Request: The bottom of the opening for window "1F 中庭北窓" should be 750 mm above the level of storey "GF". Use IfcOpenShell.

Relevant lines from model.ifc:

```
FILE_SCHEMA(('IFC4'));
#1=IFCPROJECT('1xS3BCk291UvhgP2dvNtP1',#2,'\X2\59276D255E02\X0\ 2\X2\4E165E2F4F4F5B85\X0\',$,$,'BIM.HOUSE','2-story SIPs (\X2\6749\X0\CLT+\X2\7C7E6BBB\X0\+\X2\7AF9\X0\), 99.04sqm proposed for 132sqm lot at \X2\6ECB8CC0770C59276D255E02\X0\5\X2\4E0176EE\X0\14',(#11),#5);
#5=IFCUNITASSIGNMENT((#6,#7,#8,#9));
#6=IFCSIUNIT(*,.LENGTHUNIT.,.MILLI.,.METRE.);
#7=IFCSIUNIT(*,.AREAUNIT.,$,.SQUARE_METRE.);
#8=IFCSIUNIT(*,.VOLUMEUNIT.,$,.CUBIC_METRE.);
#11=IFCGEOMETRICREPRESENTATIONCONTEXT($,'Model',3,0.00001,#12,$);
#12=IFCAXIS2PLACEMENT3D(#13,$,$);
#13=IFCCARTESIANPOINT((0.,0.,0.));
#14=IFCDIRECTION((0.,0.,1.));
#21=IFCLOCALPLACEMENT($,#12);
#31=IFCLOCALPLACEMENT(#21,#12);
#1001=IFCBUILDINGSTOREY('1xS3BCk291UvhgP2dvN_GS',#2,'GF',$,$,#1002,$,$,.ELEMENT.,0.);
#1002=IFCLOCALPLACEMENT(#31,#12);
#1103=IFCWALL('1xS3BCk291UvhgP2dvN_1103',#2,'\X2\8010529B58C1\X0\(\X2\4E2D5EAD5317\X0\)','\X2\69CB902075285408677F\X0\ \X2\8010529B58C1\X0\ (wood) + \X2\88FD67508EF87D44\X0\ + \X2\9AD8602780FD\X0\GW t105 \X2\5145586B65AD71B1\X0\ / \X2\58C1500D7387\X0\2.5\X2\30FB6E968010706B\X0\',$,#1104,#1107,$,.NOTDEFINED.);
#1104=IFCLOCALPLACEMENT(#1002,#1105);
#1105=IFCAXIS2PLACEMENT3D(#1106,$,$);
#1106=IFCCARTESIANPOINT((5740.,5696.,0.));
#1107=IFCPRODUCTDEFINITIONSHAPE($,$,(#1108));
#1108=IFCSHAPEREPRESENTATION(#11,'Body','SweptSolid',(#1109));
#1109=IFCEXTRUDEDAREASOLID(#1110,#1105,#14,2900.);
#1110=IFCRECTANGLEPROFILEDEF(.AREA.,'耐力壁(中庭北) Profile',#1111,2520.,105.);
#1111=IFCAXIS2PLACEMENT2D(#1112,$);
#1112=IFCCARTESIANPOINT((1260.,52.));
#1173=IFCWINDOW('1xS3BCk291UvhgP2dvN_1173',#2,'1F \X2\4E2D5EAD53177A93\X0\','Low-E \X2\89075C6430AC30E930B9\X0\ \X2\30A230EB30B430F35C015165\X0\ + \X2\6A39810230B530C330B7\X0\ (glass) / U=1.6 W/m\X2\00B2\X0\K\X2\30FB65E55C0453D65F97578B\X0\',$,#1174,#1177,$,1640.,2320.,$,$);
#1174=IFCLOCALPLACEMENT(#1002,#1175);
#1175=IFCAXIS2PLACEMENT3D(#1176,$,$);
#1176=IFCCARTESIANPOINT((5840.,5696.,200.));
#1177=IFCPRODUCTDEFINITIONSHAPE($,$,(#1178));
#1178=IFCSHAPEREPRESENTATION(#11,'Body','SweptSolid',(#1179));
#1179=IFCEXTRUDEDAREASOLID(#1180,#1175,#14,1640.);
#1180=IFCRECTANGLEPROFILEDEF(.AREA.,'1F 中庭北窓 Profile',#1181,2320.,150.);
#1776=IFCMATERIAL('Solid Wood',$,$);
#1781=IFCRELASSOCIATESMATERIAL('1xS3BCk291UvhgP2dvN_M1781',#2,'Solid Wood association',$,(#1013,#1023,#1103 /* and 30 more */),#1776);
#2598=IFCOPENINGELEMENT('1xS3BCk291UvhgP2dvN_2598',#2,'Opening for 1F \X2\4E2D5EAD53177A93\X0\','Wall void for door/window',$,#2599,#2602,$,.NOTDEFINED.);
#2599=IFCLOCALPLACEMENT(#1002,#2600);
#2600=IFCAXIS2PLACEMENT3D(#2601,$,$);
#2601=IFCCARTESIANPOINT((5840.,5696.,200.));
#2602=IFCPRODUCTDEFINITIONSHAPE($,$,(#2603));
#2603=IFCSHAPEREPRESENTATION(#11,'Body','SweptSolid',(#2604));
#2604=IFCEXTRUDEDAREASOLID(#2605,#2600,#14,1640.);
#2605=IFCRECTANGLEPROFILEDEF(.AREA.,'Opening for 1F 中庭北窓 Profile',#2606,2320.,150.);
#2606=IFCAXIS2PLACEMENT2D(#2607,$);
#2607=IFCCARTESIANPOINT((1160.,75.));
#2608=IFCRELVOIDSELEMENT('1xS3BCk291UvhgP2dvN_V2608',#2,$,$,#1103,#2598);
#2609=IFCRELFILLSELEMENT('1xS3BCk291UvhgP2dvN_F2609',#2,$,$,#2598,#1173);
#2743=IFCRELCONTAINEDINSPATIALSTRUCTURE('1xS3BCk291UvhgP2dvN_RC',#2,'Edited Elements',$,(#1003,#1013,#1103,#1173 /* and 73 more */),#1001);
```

```python
import numpy as np
import ifcopenshell
import ifcopenshell.api.geometry
import ifcopenshell.geom
import ifcopenshell.util.element
import ifcopenshell.util.placement
import ifcopenshell.util.shape
import ifcopenshell.util.unit

model = ifcopenshell.open("model.ifc")
unit_scale = ifcopenshell.util.unit.calculate_unit_scale(model)

window = model.by_guid("1xS3BCk291UvhgP2dvN_1173")
opening = window.FillsVoids[0].RelatingOpeningElement
storey = ifcopenshell.util.element.get_container(window, ifc_class="IfcBuildingStorey")
level = ifcopenshell.util.placement.get_local_placement(storey.ObjectPlacement)[2, 3]

# The opening's origin need not be at the sill, so measure its lowest point.
shape = ifcopenshell.geom.create_shape(ifcopenshell.geom.settings(), opening)
bottom = ifcopenshell.util.shape.get_shape_bottom_elevation(shape, shape.geometry) / unit_scale
dz = level + 0.75 / unit_scale - bottom

shift = np.array([0.0, 0.0, dz])
# The window is not placed relative to its opening, so move both.
for product in (opening, window):
    matrix = ifcopenshell.util.placement.get_local_placement(product.ObjectPlacement)
    matrix[:3, 3] += shift
    ifcopenshell.api.geometry.edit_object_placement(model, product=product, matrix=matrix, is_si=False)

print(f"moved by {dz * unit_scale:+.3f} m")

model.write("model-out.ifc")
```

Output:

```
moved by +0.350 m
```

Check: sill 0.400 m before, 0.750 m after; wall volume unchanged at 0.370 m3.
